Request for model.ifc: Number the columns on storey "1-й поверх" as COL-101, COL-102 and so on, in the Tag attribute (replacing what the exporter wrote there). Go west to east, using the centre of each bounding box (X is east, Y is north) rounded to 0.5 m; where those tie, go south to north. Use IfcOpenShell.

First a look at what the model holds.

```python
import ifcopenshell
import ifcopenshell.util.element
import ifcopenshell.util.placement

model = ifcopenshell.open("model.ifc")
print(model.schema)
storey = next(s for s in model.by_type("IfcBuildingStorey") if s.Name == "1-й поверх")
columns = [e for e in ifcopenshell.util.element.get_decomposition(storey) if e.is_a("IfcColumn")]
for e in sorted(columns, key=lambda e: e.id()):
    origin = ifcopenshell.util.placement.get_local_placement(e.ObjectPlacement)[:3, 3]
    print(e.id(), e.Tag, e.Name, origin.round(2) + 0.0, sep=" | ")
```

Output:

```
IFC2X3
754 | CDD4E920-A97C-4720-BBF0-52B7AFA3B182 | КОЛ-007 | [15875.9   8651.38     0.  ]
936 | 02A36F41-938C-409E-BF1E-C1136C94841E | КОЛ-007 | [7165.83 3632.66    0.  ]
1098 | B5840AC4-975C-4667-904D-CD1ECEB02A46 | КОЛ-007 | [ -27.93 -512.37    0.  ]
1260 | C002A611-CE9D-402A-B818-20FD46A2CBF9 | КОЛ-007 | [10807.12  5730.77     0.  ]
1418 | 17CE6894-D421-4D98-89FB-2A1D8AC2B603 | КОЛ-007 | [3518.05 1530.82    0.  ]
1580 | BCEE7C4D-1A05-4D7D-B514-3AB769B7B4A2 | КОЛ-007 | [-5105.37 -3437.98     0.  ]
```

```python
import ifcopenshell
import ifcopenshell.geom
import ifcopenshell.util.element
import ifcopenshell.util.shape

model = ifcopenshell.open("model.ifc")
settings = ifcopenshell.geom.settings()
settings.set("use-world-coords", True)


def centre(element):
    shape = ifcopenshell.geom.create_shape(settings, element)
    return ifcopenshell.util.shape.get_bbox_centroid(shape.geometry)


storey = next(s for s in model.by_type("IfcBuildingStorey") if s.Name == "1-й поверх")
columns = [e for e in ifcopenshell.util.element.get_decomposition(storey) if e.is_a("IfcColumn")]

# Insertion points can sit at a corner or the storey origin, so sort by the geometry (in metres).
centres = {e: centre(e) for e in columns}
columns.sort(key=lambda e: (round(centres[e][0] / 0.5), centres[e][1]))

for i, e in enumerate(columns, start=1):
    number = f"COL-1{i:02d}"
    e.Tag = number
    print(e.id(), number)

model.write("model-out.ifc")
```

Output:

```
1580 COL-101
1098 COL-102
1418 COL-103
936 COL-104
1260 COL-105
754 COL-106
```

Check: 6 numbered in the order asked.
